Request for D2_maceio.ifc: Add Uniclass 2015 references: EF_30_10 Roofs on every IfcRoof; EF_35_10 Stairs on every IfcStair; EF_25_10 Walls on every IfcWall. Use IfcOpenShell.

First a look at what the model holds.

```python
import ifcopenshell

model = ifcopenshell.open("D2_maceio.ifc")
print(model.schema)
print("classifications:", [c.Name for c in model.by_type("IfcClassification")])
for ifc_class in ("IfcDoor", "IfcRoof", "IfcStair", "IfcWall", "IfcWindow"):
    print(ifc_class, len(model.by_type(ifc_class)))
```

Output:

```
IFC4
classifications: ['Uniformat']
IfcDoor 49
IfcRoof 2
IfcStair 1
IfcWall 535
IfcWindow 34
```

```python
import ifcopenshell
import ifcopenshell.api.classification

model = ifcopenshell.open("D2_maceio.ifc")

system = ifcopenshell.api.classification.add_classification(model, classification="Uniclass 2015")

codes = {
    "IfcRoof": ("EF_30_10", "Roofs"),
    "IfcStair": ("EF_35_10", "Stairs"),
    "IfcWall": ("EF_25_10", "Walls"),
}
for ifc_class, (code, name) in codes.items():
    products = model.by_type(ifc_class)
    ifcopenshell.api.classification.add_reference(
        model, products=products, classification=system, identification=code, name=name
    )
    print(code, len(products))

model.write("D2_maceio_rev.ifc")
```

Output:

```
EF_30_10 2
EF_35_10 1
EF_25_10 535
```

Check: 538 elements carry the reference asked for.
